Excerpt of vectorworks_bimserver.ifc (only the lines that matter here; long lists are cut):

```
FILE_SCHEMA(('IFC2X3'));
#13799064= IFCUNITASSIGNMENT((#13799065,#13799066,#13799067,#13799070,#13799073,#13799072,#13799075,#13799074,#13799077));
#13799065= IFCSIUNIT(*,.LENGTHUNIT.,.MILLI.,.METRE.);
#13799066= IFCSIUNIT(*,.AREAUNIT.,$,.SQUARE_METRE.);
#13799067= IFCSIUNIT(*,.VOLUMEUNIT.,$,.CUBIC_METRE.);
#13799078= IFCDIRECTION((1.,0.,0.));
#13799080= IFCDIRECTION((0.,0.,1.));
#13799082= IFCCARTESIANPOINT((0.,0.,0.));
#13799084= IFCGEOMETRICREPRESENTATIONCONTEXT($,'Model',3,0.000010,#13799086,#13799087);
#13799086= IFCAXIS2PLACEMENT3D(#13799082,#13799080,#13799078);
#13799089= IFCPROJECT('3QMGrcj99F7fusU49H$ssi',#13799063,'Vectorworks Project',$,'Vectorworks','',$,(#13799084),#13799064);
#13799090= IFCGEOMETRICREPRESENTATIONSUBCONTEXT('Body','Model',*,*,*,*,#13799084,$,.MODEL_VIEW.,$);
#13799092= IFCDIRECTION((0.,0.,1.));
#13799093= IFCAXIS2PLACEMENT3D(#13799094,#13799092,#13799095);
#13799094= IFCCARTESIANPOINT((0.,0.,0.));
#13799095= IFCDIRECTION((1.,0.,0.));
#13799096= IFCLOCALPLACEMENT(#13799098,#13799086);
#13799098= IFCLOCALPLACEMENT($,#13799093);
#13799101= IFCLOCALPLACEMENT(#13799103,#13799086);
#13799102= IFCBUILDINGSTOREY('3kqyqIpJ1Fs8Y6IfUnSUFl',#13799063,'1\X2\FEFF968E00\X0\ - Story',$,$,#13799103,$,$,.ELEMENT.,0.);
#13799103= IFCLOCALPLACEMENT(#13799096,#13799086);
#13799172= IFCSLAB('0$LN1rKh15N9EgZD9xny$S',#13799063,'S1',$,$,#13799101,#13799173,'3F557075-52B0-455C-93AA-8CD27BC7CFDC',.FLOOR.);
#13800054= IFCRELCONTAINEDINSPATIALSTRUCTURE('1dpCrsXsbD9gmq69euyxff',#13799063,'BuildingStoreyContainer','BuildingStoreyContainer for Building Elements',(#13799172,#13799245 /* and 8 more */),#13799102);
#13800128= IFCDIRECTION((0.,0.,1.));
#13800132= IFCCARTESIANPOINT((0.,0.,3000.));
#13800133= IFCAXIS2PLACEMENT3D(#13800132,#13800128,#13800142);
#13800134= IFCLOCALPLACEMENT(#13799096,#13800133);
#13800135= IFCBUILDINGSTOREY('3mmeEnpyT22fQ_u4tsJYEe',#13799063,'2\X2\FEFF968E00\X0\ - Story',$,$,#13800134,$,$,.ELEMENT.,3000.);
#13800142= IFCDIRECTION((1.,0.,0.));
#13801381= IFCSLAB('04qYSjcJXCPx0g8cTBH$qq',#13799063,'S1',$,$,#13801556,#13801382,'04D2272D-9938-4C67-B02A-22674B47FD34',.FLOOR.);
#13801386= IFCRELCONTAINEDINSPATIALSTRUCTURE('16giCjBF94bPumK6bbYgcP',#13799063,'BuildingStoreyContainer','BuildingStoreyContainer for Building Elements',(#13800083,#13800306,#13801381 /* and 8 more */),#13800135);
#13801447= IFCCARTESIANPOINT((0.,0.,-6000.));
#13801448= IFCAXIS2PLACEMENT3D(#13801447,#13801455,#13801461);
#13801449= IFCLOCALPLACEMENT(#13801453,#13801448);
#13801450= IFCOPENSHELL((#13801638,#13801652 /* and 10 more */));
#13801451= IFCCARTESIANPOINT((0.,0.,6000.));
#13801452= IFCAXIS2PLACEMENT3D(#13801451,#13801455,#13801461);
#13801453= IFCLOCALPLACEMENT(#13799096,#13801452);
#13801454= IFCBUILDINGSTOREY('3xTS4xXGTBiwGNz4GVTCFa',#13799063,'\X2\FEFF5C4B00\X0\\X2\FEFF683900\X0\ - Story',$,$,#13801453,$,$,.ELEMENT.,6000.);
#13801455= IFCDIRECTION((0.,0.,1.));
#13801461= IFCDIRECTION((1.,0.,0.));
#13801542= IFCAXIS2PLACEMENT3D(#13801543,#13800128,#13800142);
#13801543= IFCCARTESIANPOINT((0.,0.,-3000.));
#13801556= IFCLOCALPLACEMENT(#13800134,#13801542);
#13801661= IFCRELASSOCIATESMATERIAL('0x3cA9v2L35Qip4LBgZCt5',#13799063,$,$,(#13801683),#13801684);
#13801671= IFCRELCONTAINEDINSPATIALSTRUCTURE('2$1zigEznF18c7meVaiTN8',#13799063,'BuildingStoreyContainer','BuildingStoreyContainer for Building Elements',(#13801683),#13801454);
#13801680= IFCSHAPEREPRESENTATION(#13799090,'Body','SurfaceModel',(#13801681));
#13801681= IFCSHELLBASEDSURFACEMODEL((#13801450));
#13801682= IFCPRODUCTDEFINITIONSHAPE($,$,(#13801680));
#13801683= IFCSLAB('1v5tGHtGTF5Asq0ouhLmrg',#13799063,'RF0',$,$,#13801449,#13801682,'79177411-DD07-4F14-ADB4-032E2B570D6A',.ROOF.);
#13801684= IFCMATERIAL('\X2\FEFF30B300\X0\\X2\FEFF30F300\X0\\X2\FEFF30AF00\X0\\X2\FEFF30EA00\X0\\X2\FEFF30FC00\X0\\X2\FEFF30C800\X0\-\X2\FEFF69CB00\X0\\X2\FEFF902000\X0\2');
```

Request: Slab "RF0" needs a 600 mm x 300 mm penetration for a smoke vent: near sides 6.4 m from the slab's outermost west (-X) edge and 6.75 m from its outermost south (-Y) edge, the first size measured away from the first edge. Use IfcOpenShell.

```python
import numpy as np
import ifcopenshell
import ifcopenshell.api.feature
import ifcopenshell.api.geometry
import ifcopenshell.api.root
import ifcopenshell.geom
import ifcopenshell.util.placement
import ifcopenshell.util.representation
import ifcopenshell.util.shape
import ifcopenshell.util.unit

model = ifcopenshell.open("vectorworks_bimserver.ifc")
unit_scale = ifcopenshell.util.unit.calculate_unit_scale(model)
settings = ifcopenshell.geom.settings()


def volume(element):
    """Net volume in cubic metres, openings subtracted."""
    shape = ifcopenshell.geom.create_shape(settings, element)
    return ifcopenshell.util.shape.get_volume(shape.geometry)


slab = model.by_guid("1v5tGHtGTF5Asq0ouhLmrg")
before = volume(slab)

# Extent in the slab's own axes, in metres. The edges named are its -X and -Y sides.
slab_shape = ifcopenshell.geom.create_shape(settings, slab)
vertices = ifcopenshell.util.shape.get_vertices(slab_shape.geometry)
x_min, y_min, bottom = vertices.min(axis=0)
top = vertices[:, 2].max()

opening = ifcopenshell.api.root.create_entity(model, ifc_class="IfcOpeningElement", name="Smoke vent opening")
context = ifcopenshell.util.representation.get_context(model, "Model", "Body", "MODEL_VIEW")
width, depth = 0.6, 0.3
outline = [(0.0, 0.0), (width, 0.0), (width, depth), (0.0, depth), (0.0, 0.0)]
# Overshoot both faces by 50 mm so the cut is clean.
shape = ifcopenshell.api.geometry.add_slab_representation(
    model, context=context, depth=top - bottom + 0.1, polyline=outline
)
ifcopenshell.api.geometry.assign_representation(model, product=opening, representation=shape)

matrix = ifcopenshell.util.placement.get_local_placement(slab.ObjectPlacement)
matrix[:, 3] = matrix @ np.append(np.array([x_min + 6.4, y_min + 6.75, bottom - 0.05]) / unit_scale, 1.0)
ifcopenshell.api.geometry.edit_object_placement(model, product=opening, matrix=matrix, is_si=False)
ifcopenshell.api.feature.add_feature(model, feature=opening, element=slab)

after = volume(slab)

print(f"slab volume {before:.3f} -> {after:.3f} m3")

model.write("vectorworks_bimserver_edited.ifc")
```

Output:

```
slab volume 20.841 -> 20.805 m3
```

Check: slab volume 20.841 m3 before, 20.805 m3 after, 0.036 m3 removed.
